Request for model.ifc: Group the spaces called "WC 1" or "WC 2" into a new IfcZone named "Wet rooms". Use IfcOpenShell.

First a look at what the model holds.

```python
import ifcopenshell

model = ifcopenshell.open("model.ifc")
print(model.schema)
seen = {}
for space in model.by_type("IfcSpace"):
    seen[space.LongName] = seen.get(space.LongName, 0) + 1
for name, count in sorted(seen.items(), key=str):
    print(count, "x", name)
print("zones:", [z.Name for z in model.by_type("IfcZone")][:20])
```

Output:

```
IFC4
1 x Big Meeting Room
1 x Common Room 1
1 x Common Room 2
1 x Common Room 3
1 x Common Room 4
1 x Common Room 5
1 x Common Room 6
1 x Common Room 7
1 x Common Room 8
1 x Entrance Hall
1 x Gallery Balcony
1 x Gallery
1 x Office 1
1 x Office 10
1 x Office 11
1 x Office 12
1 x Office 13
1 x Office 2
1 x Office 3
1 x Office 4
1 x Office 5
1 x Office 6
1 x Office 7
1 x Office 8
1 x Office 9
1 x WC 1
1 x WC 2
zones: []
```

```python
import ifcopenshell
import ifcopenshell.api.group
import ifcopenshell.api.root

model = ifcopenshell.open("model.ifc")

names = {"WC 1", "WC 2"}
spaces = [s for s in model.by_type("IfcSpace") if s.LongName in names]

zone = ifcopenshell.api.root.create_entity(model, ifc_class="IfcZone", name="Wet rooms")
ifcopenshell.api.group.assign_group(model, products=spaces, group=zone)
print(len(spaces), "spaces in", zone.Name)

model.write("model_edited.ifc")
```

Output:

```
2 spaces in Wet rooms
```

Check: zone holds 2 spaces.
